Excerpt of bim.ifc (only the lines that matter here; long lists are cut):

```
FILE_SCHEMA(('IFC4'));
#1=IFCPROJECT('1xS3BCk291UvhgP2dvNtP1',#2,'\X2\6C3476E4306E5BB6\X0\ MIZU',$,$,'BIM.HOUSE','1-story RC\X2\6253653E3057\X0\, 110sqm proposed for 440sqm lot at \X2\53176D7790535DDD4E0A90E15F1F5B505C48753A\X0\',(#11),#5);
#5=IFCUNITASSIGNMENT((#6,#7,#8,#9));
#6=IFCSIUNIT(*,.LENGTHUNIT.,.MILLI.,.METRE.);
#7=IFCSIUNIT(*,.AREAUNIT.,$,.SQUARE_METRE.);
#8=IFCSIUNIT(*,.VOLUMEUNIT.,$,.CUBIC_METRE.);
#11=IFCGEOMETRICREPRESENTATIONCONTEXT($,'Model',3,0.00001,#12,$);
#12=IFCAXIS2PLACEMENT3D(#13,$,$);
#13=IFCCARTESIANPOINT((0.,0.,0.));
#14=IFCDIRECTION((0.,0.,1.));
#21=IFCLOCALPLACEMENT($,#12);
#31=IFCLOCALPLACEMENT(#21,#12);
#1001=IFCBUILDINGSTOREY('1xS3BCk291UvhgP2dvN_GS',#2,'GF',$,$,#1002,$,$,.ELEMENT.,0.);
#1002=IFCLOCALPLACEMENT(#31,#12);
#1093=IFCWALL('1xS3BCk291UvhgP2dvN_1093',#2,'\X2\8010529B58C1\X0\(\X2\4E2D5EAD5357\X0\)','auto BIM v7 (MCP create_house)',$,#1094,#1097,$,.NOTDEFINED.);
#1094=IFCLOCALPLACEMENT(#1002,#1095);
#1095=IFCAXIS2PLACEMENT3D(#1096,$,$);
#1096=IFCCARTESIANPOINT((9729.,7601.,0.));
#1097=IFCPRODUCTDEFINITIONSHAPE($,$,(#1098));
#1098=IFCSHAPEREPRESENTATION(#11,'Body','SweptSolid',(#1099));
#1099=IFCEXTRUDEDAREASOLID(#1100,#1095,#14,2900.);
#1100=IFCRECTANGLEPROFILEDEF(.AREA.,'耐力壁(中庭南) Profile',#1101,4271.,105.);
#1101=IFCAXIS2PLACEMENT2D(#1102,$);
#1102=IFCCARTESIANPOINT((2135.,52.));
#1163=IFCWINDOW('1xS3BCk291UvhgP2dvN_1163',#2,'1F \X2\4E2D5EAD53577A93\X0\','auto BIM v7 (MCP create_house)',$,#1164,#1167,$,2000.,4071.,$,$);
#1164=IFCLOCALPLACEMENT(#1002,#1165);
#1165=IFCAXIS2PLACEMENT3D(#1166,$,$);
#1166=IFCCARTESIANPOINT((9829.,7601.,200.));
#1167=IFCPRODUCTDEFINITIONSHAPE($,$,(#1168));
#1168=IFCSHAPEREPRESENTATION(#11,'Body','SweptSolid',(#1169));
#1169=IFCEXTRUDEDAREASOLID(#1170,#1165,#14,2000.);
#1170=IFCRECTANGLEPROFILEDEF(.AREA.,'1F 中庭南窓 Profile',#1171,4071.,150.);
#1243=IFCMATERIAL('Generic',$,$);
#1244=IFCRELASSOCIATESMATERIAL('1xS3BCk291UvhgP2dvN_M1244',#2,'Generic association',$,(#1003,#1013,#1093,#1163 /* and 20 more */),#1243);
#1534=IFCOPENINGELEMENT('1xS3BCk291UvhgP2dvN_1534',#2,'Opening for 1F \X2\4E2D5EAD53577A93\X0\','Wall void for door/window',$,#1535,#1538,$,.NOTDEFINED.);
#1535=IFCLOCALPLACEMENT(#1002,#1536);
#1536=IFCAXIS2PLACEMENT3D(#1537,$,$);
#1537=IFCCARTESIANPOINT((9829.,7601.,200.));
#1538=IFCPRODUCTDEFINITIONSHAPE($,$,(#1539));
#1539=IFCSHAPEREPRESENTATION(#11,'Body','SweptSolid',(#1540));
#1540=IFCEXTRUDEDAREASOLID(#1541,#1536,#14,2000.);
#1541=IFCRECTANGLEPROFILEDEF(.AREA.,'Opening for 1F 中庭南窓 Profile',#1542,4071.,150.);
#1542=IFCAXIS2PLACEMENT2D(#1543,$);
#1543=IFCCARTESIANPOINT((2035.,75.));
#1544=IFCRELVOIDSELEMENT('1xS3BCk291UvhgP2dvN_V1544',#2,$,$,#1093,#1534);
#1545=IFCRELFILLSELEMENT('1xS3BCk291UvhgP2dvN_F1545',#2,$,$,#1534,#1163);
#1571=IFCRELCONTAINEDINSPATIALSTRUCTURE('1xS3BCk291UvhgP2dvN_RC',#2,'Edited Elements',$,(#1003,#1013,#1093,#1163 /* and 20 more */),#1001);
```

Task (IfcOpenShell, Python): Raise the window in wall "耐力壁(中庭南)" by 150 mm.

```python
import numpy as np
import ifcopenshell
import ifcopenshell.api.geometry
import ifcopenshell.util.placement
import ifcopenshell.util.unit

model = ifcopenshell.open("bim.ifc")
unit_scale = ifcopenshell.util.unit.calculate_unit_scale(model)

window = model.by_guid("1xS3BCk291UvhgP2dvN_1163")
opening = window.FillsVoids[0].RelatingOpeningElement
dz = 150.0

shift = np.array([0.0, 0.0, dz])
# The window is not placed relative to its opening, so move both.
for product in (opening, window):
    matrix = ifcopenshell.util.placement.get_local_placement(product.ObjectPlacement)
    matrix[:3, 3] += shift
    ifcopenshell.api.geometry.edit_object_placement(model, product=product, matrix=matrix, is_si=False)

print(f"moved by {dz * unit_scale:+.3f} m")

model.write("bim_rev.ifc")
```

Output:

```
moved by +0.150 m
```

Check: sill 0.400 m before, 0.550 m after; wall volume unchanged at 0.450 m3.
